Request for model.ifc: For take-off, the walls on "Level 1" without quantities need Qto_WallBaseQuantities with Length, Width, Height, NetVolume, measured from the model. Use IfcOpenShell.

First a look at what the model holds.

```python
import ifcopenshell
import ifcopenshell.util.element
import ifcopenshell.util.unit

model = ifcopenshell.open("model.ifc")
print(model.schema)
for unit_type in ("LENGTHUNIT", "AREAUNIT", "VOLUMEUNIT"):
    print(unit_type, ifcopenshell.util.unit.calculate_unit_scale(model, unit_type))
storey = next(s for s in model.by_type("IfcBuildingStorey") if s.Name == "Level 1")
walls = [e for e in ifcopenshell.util.element.get_decomposition(storey) if e.is_a("IfcWall")]
for e in sorted(walls, key=lambda e: e.id()):
    print(e.id(), e.is_a(), e.Name, list(ifcopenshell.util.element.get_psets(e, qtos_only=True)), sep=" | ")
```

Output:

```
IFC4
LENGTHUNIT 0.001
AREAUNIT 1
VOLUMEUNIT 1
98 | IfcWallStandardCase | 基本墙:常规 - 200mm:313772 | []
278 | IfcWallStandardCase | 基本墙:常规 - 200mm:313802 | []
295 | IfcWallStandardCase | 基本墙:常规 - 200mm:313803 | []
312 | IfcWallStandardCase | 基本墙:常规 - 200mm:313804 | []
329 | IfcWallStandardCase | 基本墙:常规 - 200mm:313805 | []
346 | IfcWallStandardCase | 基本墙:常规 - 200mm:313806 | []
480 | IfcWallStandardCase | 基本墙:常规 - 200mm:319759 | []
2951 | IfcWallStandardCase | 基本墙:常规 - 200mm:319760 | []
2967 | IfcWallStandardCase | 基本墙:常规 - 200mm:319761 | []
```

```python
import ifcopenshell
import ifcopenshell.api.pset
import ifcopenshell.geom
import ifcopenshell.util.element
import ifcopenshell.util.shape
import ifcopenshell.util.unit

model = ifcopenshell.open("model.ifc")
unit_scale = ifcopenshell.util.unit.calculate_unit_scale(model)
volume_scale = ifcopenshell.util.unit.calculate_unit_scale(model, "VOLUMEUNIT")
settings = ifcopenshell.geom.settings()

storey = next(s for s in model.by_type("IfcBuildingStorey") if s.Name == "Level 1")
walls = [e for e in ifcopenshell.util.element.get_decomposition(storey) if e.is_a("IfcWall")]

for e in sorted(walls, key=lambda e: e.id()):
    if ifcopenshell.util.element.get_psets(e, qtos_only=True, should_inherit=False):
        continue
    # Geometry comes back in metres, in the element's own axes.
    shape = ifcopenshell.geom.create_shape(settings, e)
    values = {
        "Length": ifcopenshell.util.shape.get_x(shape.geometry) / unit_scale,
        "Width": ifcopenshell.util.shape.get_y(shape.geometry) / unit_scale,
        "Height": ifcopenshell.util.shape.get_z(shape.geometry) / unit_scale,
        "NetVolume": ifcopenshell.util.shape.get_volume(shape.geometry) / volume_scale,
    }
    qto = ifcopenshell.api.pset.add_qto(model, product=e, name="Qto_WallBaseQuantities")
    ifcopenshell.api.pset.edit_qto(model, qto=qto, properties=values)
    print(e.id(), {k: round(v, 3) for k, v in values.items()})

model.write("model_updated.ifc")
```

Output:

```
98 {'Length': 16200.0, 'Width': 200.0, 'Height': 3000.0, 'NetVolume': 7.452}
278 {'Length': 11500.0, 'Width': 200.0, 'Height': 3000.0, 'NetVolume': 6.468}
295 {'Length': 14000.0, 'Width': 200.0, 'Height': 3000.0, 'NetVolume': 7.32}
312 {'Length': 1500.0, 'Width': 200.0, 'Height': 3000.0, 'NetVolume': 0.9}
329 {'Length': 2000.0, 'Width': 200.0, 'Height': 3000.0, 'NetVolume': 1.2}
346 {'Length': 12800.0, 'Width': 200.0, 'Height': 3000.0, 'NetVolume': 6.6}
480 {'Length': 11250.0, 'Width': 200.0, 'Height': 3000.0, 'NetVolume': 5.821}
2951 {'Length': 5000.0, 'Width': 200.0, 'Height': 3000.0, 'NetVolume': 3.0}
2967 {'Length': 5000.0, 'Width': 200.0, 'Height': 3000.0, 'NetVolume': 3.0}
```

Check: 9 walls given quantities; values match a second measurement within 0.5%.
